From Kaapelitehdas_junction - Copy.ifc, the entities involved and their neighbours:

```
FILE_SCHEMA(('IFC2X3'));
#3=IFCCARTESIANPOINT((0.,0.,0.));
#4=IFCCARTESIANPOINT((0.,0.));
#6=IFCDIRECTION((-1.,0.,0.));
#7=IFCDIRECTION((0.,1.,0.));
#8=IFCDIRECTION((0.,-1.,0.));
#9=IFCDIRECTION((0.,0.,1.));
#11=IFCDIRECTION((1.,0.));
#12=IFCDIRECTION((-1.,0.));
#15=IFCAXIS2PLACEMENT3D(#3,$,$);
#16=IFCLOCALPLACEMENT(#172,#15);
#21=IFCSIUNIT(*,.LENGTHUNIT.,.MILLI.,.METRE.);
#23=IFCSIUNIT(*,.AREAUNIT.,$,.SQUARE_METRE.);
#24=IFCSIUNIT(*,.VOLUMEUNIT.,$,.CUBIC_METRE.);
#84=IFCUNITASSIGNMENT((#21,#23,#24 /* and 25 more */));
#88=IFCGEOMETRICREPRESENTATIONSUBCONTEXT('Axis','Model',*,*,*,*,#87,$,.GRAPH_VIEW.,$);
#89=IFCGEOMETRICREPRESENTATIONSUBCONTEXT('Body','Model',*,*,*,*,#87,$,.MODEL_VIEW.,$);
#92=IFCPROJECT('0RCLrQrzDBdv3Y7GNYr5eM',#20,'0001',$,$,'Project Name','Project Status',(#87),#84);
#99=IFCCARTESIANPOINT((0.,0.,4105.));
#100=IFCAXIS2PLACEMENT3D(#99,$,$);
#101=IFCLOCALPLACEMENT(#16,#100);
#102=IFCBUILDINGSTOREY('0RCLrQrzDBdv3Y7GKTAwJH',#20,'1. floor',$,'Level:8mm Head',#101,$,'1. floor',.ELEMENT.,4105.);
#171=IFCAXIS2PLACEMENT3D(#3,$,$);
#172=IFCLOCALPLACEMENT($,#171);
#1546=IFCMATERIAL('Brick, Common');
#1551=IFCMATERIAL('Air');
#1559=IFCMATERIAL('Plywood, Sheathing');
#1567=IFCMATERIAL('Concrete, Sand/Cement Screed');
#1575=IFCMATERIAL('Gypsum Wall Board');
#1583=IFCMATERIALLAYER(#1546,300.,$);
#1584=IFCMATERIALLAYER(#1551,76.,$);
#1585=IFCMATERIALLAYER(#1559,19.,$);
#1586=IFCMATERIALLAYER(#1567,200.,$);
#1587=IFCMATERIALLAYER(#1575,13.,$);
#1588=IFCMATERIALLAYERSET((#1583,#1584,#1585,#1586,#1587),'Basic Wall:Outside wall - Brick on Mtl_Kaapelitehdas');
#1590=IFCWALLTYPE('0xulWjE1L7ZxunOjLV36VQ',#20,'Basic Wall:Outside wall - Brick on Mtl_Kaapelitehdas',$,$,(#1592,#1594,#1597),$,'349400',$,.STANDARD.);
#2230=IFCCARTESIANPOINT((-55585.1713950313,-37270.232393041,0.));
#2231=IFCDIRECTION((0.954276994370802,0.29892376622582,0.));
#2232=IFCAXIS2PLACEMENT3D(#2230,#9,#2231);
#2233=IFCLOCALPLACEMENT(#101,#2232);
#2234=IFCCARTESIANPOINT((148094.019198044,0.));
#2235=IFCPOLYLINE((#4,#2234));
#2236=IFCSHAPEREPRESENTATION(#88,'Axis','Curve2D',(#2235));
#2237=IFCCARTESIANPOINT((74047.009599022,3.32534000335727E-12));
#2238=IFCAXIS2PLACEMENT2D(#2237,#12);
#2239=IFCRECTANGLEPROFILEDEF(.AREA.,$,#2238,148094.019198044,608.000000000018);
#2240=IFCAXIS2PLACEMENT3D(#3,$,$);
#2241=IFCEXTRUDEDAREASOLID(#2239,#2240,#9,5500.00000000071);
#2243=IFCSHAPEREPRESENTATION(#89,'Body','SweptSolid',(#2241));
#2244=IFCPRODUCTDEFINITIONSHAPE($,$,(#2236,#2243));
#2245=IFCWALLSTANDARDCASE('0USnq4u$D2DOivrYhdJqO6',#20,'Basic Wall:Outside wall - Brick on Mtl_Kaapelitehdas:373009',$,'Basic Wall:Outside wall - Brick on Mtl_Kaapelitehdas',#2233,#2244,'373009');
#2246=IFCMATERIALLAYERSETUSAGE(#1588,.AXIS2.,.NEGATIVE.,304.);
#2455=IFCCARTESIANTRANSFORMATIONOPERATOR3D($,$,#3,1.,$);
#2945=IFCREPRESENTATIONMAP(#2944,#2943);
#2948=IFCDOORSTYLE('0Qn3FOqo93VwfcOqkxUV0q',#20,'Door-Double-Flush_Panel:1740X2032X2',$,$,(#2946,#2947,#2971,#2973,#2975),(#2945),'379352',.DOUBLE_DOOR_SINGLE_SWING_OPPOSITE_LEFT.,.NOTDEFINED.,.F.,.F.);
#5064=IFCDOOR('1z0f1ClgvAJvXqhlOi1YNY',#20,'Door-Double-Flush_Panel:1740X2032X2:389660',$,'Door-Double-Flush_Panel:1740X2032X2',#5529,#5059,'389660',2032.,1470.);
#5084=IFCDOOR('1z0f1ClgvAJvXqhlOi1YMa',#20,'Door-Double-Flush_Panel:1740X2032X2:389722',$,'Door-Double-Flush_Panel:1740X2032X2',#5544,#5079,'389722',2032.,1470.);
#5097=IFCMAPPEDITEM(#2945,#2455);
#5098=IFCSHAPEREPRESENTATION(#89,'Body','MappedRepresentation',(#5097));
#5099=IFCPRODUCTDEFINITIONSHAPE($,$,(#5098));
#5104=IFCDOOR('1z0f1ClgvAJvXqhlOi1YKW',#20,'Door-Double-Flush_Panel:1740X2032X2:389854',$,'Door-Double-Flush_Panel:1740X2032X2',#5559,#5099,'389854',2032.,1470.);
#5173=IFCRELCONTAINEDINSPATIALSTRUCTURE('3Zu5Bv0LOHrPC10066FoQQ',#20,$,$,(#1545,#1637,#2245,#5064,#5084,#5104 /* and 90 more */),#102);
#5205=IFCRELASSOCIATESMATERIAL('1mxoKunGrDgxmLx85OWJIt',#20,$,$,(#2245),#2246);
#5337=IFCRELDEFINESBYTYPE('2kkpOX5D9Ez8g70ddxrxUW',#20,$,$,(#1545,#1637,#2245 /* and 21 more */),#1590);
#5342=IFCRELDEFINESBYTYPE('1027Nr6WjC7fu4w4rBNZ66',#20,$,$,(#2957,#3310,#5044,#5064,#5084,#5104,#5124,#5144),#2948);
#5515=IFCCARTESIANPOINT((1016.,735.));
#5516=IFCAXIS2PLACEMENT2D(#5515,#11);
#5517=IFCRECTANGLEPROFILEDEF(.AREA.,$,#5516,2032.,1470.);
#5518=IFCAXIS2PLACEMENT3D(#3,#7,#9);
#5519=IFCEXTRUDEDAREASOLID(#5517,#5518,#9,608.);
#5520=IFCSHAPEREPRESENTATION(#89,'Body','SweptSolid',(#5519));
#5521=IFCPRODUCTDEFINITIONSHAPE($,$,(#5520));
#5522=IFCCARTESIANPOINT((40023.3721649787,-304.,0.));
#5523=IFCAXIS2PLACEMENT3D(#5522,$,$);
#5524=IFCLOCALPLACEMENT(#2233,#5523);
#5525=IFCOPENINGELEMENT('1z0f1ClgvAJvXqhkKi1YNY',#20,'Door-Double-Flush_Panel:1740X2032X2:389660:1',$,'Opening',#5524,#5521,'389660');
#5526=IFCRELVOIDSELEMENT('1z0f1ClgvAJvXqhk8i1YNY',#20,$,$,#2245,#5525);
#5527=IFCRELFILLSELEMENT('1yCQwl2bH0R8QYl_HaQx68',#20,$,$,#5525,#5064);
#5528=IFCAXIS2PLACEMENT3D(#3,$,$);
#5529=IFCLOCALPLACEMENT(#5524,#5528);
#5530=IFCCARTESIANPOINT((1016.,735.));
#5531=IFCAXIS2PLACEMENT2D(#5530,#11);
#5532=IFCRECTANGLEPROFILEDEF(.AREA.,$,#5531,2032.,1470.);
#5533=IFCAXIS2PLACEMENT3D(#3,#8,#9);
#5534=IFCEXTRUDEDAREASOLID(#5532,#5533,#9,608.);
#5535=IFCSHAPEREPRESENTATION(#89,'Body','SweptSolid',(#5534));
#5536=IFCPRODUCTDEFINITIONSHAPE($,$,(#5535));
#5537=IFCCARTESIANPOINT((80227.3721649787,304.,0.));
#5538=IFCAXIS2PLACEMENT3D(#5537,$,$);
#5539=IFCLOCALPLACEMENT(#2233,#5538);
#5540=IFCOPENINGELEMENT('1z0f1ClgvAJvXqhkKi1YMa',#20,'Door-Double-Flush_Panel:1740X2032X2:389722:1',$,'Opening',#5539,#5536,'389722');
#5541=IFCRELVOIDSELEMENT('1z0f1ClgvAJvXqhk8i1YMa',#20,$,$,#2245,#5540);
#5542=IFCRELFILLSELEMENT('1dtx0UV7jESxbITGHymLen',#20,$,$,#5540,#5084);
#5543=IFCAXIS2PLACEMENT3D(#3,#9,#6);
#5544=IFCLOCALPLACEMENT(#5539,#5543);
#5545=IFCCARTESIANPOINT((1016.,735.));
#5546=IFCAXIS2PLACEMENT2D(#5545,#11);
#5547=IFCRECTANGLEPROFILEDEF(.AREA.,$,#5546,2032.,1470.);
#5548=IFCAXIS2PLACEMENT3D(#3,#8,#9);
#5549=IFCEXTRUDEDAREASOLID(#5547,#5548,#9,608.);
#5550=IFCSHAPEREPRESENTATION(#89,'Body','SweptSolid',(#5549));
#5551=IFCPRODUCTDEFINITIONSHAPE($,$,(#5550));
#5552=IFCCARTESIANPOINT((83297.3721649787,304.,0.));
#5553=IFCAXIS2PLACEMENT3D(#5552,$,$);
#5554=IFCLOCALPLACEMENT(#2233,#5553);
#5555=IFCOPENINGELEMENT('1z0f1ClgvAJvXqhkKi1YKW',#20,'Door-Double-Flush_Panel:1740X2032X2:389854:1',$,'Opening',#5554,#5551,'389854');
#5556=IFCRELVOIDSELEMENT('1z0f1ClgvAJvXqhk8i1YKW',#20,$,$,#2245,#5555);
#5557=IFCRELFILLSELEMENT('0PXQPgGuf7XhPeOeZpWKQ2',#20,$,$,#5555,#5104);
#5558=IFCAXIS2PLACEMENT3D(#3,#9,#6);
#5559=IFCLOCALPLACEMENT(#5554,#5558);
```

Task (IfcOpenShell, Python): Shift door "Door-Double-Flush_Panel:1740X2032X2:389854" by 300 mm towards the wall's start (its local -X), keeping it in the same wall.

```python
import ifcopenshell
import ifcopenshell.api.geometry
import ifcopenshell.util.placement
import ifcopenshell.util.unit

model = ifcopenshell.open("Kaapelitehdas_junction - Copy.ifc")
unit_scale = ifcopenshell.util.unit.calculate_unit_scale(model)

door = model.by_guid("1z0f1ClgvAJvXqhlOi1YKW")
opening = door.FillsVoids[0].RelatingOpeningElement
wall = opening.VoidsElements[0].RelatingBuildingElement

wall_matrix = ifcopenshell.util.placement.get_local_placement(wall.ObjectPlacement)
shift = wall_matrix[:3, 0] * -0.3 / unit_scale
before = ifcopenshell.util.placement.get_local_placement(door.ObjectPlacement)[:3, 3].copy()

# The door is placed relative to its opening, so it follows when the opening moves.
matrix = ifcopenshell.util.placement.get_local_placement(opening.ObjectPlacement)
matrix[:3, 3] += shift
ifcopenshell.api.geometry.edit_object_placement(
    model, product=opening, matrix=matrix, is_si=False, should_transform_children=True
)

after = ifcopenshell.util.placement.get_local_placement(door.ObjectPlacement)[:3, 3]
print("door moved by", (after - before).round(3) + 0.0)

model.write("Kaapelitehdas_junction - Copy-out.ifc")
```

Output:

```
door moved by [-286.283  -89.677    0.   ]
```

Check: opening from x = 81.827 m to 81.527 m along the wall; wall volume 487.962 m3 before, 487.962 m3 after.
